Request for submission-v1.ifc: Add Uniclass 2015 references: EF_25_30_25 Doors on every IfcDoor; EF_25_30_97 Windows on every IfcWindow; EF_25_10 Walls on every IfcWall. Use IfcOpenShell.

First a look at what the model holds.

```python
import ifcopenshell

model = ifcopenshell.open("submission-v1.ifc")
print(model.schema)
print("classifications:", [c.Name for c in model.by_type("IfcClassification")])
for ifc_class in ("IfcDoor", "IfcRoof", "IfcStair", "IfcWall", "IfcWindow"):
    print(ifc_class, len(model.by_type(ifc_class)))
```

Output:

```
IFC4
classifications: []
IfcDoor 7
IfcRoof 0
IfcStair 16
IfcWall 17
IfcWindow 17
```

```python
import ifcopenshell
import ifcopenshell.api.classification

model = ifcopenshell.open("submission-v1.ifc")

system = ifcopenshell.api.classification.add_classification(model, classification="Uniclass 2015")

codes = {
    "IfcDoor": ("EF_25_30_25", "Doors"),
    "IfcWindow": ("EF_25_30_97", "Windows"),
    "IfcWall": ("EF_25_10", "Walls"),
}
for ifc_class, (code, name) in codes.items():
    products = model.by_type(ifc_class)
    ifcopenshell.api.classification.add_reference(
        model, products=products, classification=system, identification=code, name=name
    )
    print(code, len(products))

model.write("submission-v1_updated.ifc")
```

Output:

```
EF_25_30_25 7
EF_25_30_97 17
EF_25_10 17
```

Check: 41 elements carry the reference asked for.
